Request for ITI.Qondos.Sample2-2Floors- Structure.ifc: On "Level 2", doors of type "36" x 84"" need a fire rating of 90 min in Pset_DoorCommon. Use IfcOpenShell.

First a look at what the model holds.

```python
import ifcopenshell
import ifcopenshell.util.element

model = ifcopenshell.open("ITI.Qondos.Sample2-2Floors- Structure.ifc")
print(model.schema)
storey = next(s for s in model.by_type("IfcBuildingStorey") if s.Name == "Level 2")
doors = [e for e in ifcopenshell.util.element.get_decomposition(storey) if e.is_a("IfcDoor")]
seen = {}
for e in doors:
    element_type = ifcopenshell.util.element.get_type(e)
    key = (element_type.Name if element_type != e and element_type else None, ifcopenshell.util.element.get_pset(e, "Pset_DoorCommon", "FireRating"))
    seen[key] = seen.get(key, 0) + 1
for (name, value), count in sorted(seen.items(), key=str):
    print(count, "x", name, "|", value)
```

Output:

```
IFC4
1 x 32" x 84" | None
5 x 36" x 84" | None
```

```python
import ifcopenshell
import ifcopenshell.api.pset
import ifcopenshell.util.element

model = ifcopenshell.open("ITI.Qondos.Sample2-2Floors- Structure.ifc")

storey = next(s for s in model.by_type("IfcBuildingStorey") if s.Name == "Level 2")
doors = [e for e in ifcopenshell.util.element.get_decomposition(storey) if e.is_a("IfcDoor")]

count = 0
for e in doors:
    element_type = ifcopenshell.util.element.get_type(e)
    if element_type in (None, e) or element_type.Name != '36" x 84"':
        continue
    # add_pset returns the element's existing set when there is one.
    pset = ifcopenshell.api.pset.add_pset(model, product=e, name="Pset_DoorCommon")
    ifcopenshell.api.pset.edit_pset(model, pset=pset, properties={"FireRating": "90 min"})
    count += 1

print(count, "doors updated")

model.write("ITI.Qondos.Sample2-2Floors- Structure-out.ifc")
```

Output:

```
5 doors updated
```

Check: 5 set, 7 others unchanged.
